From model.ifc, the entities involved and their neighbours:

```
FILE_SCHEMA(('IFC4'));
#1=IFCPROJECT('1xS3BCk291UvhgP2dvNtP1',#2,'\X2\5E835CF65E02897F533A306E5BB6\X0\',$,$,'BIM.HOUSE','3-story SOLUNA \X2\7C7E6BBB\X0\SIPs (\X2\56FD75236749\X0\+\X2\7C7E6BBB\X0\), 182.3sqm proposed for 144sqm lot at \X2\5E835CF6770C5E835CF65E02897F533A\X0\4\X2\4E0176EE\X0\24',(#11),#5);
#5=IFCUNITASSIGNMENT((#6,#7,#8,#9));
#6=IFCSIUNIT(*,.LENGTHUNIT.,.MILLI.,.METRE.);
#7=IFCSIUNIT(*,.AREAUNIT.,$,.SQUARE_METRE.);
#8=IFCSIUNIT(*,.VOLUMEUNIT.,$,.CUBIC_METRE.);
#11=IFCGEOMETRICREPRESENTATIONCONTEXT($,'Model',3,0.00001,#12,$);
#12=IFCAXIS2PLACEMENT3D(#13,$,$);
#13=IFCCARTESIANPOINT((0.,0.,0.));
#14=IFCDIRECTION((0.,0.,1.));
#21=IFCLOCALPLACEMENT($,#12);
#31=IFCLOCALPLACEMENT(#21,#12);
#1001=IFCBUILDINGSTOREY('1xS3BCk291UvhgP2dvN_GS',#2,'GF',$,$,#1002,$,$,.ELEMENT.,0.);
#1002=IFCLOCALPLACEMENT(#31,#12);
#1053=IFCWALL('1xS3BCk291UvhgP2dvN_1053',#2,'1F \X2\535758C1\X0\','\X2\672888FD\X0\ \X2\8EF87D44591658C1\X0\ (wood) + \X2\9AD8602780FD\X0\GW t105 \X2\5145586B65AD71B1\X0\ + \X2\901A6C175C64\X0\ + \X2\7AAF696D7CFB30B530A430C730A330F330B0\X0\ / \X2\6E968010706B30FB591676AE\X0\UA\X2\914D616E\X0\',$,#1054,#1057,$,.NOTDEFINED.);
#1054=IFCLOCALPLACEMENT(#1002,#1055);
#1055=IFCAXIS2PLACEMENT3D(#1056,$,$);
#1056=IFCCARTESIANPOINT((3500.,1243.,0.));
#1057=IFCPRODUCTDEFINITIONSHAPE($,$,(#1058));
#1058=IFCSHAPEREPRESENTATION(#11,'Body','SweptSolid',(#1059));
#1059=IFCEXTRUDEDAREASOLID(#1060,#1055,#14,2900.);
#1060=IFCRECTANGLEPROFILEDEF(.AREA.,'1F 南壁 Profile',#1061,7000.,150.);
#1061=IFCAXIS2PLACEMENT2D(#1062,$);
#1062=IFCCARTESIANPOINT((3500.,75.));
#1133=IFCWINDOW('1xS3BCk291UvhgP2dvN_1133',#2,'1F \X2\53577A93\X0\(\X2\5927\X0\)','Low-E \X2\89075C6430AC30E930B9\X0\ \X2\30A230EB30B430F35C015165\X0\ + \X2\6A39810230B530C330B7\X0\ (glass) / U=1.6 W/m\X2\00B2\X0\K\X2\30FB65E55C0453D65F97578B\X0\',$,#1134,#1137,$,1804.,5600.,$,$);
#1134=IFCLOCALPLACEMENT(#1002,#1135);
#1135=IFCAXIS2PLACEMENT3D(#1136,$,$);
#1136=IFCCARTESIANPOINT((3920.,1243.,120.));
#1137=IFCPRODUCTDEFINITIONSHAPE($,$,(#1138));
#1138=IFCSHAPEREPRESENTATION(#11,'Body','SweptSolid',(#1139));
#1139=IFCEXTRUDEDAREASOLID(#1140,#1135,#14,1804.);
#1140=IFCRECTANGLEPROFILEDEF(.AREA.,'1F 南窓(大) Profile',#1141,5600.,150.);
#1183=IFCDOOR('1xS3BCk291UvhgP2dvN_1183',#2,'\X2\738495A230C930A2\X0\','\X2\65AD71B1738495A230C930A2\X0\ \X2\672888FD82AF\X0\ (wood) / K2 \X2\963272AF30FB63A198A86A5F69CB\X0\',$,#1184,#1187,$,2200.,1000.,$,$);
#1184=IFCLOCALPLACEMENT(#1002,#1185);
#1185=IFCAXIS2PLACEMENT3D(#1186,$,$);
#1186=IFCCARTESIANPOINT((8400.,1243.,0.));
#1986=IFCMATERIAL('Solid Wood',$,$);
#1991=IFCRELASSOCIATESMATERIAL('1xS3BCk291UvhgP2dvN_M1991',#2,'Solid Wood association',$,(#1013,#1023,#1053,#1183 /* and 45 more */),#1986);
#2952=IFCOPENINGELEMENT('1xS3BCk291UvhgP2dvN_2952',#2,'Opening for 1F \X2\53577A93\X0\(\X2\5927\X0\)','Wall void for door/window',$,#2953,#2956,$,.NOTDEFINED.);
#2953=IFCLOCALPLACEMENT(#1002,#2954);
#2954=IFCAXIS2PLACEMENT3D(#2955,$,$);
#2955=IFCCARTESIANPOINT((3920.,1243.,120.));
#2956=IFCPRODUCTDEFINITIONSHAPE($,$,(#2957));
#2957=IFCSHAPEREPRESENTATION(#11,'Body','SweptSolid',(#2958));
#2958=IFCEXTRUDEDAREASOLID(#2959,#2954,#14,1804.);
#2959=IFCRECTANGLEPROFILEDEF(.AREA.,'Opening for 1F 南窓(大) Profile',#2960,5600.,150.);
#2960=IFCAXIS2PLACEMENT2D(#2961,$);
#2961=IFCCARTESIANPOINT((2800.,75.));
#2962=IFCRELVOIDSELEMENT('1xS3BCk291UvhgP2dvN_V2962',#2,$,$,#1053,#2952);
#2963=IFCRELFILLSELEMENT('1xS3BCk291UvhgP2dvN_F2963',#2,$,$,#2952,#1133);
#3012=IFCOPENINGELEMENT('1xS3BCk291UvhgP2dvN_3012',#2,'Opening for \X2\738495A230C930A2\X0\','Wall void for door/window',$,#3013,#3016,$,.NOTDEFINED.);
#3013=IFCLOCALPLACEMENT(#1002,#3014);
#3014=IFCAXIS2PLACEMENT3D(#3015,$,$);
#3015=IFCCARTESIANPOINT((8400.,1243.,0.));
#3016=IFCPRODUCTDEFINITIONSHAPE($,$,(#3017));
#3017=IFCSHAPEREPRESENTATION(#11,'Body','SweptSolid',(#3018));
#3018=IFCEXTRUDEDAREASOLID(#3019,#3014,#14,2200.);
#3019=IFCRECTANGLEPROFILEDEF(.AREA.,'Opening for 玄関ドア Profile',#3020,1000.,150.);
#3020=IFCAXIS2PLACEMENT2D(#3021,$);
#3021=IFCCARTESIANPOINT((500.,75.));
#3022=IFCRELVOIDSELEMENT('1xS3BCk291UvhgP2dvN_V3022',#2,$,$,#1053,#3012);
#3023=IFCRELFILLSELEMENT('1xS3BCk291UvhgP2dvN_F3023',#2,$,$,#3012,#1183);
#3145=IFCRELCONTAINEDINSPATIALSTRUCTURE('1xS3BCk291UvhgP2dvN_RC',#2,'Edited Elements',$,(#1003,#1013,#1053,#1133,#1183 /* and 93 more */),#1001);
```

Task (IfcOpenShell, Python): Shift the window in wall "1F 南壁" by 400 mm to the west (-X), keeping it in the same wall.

```python
import ifcopenshell
import ifcopenshell.api.geometry
import ifcopenshell.util.placement
import ifcopenshell.util.unit

model = ifcopenshell.open("model.ifc")
unit_scale = ifcopenshell.util.unit.calculate_unit_scale(model)

window = model.by_guid("1xS3BCk291UvhgP2dvN_1133")
opening = window.FillsVoids[0].RelatingOpeningElement
wall = opening.VoidsElements[0].RelatingBuildingElement

wall_matrix = ifcopenshell.util.placement.get_local_placement(wall.ObjectPlacement)
shift = wall_matrix[:3, 0] * -0.4 / unit_scale
before = ifcopenshell.util.placement.get_local_placement(window.ObjectPlacement)[:3, 3].copy()

# The window is not placed relative to its opening, so move both.
for product in (opening, window):
    matrix = ifcopenshell.util.placement.get_local_placement(product.ObjectPlacement)
    matrix[:3, 3] += shift
    ifcopenshell.api.geometry.edit_object_placement(model, product=product, matrix=matrix, is_si=False)

after = ifcopenshell.util.placement.get_local_placement(window.ObjectPlacement)[:3, 3]
print("window moved by", (after - before).round(3) + 0.0)

model.write("model_v2.ifc")
```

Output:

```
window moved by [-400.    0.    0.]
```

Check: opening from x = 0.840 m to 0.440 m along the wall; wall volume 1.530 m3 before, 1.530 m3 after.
